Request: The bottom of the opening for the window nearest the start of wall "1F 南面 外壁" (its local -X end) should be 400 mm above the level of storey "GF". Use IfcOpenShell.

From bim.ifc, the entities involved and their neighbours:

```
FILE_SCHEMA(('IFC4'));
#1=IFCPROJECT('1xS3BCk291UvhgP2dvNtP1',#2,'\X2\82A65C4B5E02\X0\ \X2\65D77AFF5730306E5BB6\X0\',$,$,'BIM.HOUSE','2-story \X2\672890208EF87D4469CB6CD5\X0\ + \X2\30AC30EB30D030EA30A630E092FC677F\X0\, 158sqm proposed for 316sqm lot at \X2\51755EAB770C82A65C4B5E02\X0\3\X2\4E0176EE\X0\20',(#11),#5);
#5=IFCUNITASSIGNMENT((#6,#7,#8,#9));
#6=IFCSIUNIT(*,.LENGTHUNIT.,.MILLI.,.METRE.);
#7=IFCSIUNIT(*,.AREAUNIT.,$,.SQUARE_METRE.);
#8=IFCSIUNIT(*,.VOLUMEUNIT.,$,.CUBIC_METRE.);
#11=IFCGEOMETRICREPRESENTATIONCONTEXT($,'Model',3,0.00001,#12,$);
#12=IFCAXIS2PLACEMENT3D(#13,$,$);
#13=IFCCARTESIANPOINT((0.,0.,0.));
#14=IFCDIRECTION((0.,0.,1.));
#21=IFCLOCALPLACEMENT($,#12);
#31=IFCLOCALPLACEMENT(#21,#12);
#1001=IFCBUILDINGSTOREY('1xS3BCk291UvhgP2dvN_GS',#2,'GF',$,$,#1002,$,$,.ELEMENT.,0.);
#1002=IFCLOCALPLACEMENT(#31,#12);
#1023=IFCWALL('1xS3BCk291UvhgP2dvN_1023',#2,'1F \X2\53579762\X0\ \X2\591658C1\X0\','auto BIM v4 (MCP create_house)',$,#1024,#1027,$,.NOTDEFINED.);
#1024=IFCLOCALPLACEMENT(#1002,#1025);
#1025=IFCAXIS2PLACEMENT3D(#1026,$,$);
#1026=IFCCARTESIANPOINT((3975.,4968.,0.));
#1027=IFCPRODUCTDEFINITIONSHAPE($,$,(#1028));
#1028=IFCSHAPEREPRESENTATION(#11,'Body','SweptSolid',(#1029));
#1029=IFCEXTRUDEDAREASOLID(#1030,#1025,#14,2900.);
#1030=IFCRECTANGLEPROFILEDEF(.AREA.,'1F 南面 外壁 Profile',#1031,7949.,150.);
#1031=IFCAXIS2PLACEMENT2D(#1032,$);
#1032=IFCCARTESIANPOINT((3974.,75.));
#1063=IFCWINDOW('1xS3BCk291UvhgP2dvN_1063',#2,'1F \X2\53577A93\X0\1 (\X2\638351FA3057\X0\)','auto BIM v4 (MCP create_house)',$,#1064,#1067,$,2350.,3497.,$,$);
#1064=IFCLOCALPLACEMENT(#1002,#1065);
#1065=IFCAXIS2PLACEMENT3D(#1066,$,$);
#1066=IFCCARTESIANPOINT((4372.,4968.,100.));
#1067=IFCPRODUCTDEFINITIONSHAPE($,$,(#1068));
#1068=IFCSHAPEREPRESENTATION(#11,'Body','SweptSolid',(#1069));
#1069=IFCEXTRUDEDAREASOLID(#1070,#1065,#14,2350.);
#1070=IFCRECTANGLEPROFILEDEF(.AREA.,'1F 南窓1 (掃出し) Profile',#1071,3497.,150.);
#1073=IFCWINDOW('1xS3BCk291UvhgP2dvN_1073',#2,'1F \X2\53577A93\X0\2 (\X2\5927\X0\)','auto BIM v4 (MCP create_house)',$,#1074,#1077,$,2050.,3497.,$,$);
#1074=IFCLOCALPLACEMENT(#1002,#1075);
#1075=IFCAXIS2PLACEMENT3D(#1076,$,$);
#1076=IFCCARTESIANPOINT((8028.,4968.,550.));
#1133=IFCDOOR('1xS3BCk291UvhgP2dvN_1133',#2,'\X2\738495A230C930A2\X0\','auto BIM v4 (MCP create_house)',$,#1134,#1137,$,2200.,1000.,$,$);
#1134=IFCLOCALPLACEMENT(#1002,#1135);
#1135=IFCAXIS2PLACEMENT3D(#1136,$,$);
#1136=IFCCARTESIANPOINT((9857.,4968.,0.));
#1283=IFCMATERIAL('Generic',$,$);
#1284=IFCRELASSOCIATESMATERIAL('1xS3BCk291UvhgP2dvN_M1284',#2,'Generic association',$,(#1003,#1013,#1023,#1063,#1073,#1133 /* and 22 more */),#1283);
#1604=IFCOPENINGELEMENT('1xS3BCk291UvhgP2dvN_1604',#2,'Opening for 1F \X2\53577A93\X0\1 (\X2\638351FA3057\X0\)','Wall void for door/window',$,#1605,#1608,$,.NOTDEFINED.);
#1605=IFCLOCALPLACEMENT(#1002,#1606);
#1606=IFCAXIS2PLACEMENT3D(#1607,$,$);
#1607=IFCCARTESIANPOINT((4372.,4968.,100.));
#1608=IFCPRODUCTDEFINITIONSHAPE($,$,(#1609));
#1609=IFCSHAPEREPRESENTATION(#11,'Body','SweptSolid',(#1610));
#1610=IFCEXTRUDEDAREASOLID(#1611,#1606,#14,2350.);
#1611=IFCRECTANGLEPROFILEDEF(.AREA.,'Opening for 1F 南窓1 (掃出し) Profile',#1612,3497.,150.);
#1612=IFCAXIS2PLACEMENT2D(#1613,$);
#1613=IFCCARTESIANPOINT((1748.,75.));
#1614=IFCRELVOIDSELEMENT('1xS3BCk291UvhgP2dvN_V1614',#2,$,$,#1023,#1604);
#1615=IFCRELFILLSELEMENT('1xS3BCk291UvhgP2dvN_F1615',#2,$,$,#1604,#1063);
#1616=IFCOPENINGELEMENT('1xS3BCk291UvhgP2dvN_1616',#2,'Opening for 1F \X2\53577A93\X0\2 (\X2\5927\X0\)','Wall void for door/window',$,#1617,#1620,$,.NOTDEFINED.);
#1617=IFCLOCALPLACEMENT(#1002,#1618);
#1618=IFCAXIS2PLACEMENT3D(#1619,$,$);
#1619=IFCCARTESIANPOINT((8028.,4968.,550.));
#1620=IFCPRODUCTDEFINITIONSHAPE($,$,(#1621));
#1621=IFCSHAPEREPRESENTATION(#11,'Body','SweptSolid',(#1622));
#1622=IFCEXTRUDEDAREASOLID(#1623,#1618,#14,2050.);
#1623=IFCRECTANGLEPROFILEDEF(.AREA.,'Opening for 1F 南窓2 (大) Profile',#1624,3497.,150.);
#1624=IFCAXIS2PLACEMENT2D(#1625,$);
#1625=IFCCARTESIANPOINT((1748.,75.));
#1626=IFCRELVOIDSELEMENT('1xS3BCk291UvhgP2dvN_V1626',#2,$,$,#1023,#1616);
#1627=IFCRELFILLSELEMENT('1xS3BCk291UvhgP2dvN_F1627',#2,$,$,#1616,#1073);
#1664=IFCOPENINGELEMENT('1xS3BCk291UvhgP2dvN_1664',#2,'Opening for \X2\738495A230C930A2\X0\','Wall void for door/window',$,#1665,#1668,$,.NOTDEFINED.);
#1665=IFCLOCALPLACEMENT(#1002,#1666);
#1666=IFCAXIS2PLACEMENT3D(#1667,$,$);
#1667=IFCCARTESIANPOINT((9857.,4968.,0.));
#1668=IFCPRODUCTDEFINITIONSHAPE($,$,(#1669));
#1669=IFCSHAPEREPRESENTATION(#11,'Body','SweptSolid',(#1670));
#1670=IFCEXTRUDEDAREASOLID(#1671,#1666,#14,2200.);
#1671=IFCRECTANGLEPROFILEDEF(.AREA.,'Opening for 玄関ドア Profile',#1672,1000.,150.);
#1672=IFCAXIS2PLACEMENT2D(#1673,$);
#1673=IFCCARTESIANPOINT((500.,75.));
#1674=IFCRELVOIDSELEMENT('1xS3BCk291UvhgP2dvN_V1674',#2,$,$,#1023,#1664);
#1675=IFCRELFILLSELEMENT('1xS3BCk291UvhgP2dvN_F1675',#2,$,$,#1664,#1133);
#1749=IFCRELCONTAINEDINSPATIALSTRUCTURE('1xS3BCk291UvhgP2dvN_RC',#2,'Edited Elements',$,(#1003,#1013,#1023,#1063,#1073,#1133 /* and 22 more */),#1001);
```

```python
import numpy as np
import ifcopenshell
import ifcopenshell.api.geometry
import ifcopenshell.geom
import ifcopenshell.util.element
import ifcopenshell.util.placement
import ifcopenshell.util.shape
import ifcopenshell.util.unit

model = ifcopenshell.open("bim.ifc")
unit_scale = ifcopenshell.util.unit.calculate_unit_scale(model)

window = model.by_id(1063)
opening = window.FillsVoids[0].RelatingOpeningElement
storey = ifcopenshell.util.element.get_container(window, ifc_class="IfcBuildingStorey")
level = ifcopenshell.util.placement.get_local_placement(storey.ObjectPlacement)[2, 3]

# The opening's origin need not be at the sill, so measure its lowest point.
shape = ifcopenshell.geom.create_shape(ifcopenshell.geom.settings(), opening)
bottom = ifcopenshell.util.shape.get_shape_bottom_elevation(shape, shape.geometry) / unit_scale
dz = level + 400.0 - bottom

shift = np.array([0.0, 0.0, dz])
# The window is not placed relative to its opening, so move both.
for product in (opening, window):
    matrix = ifcopenshell.util.placement.get_local_placement(product.ObjectPlacement)
    matrix[:3, 3] += shift
    ifcopenshell.api.geometry.edit_object_placement(model, product=product, matrix=matrix, is_si=False)

print(f"moved by {dz * unit_scale:+.3f} m")

model.write("bim-out.ifc")
```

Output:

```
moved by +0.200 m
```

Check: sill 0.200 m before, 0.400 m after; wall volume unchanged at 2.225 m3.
